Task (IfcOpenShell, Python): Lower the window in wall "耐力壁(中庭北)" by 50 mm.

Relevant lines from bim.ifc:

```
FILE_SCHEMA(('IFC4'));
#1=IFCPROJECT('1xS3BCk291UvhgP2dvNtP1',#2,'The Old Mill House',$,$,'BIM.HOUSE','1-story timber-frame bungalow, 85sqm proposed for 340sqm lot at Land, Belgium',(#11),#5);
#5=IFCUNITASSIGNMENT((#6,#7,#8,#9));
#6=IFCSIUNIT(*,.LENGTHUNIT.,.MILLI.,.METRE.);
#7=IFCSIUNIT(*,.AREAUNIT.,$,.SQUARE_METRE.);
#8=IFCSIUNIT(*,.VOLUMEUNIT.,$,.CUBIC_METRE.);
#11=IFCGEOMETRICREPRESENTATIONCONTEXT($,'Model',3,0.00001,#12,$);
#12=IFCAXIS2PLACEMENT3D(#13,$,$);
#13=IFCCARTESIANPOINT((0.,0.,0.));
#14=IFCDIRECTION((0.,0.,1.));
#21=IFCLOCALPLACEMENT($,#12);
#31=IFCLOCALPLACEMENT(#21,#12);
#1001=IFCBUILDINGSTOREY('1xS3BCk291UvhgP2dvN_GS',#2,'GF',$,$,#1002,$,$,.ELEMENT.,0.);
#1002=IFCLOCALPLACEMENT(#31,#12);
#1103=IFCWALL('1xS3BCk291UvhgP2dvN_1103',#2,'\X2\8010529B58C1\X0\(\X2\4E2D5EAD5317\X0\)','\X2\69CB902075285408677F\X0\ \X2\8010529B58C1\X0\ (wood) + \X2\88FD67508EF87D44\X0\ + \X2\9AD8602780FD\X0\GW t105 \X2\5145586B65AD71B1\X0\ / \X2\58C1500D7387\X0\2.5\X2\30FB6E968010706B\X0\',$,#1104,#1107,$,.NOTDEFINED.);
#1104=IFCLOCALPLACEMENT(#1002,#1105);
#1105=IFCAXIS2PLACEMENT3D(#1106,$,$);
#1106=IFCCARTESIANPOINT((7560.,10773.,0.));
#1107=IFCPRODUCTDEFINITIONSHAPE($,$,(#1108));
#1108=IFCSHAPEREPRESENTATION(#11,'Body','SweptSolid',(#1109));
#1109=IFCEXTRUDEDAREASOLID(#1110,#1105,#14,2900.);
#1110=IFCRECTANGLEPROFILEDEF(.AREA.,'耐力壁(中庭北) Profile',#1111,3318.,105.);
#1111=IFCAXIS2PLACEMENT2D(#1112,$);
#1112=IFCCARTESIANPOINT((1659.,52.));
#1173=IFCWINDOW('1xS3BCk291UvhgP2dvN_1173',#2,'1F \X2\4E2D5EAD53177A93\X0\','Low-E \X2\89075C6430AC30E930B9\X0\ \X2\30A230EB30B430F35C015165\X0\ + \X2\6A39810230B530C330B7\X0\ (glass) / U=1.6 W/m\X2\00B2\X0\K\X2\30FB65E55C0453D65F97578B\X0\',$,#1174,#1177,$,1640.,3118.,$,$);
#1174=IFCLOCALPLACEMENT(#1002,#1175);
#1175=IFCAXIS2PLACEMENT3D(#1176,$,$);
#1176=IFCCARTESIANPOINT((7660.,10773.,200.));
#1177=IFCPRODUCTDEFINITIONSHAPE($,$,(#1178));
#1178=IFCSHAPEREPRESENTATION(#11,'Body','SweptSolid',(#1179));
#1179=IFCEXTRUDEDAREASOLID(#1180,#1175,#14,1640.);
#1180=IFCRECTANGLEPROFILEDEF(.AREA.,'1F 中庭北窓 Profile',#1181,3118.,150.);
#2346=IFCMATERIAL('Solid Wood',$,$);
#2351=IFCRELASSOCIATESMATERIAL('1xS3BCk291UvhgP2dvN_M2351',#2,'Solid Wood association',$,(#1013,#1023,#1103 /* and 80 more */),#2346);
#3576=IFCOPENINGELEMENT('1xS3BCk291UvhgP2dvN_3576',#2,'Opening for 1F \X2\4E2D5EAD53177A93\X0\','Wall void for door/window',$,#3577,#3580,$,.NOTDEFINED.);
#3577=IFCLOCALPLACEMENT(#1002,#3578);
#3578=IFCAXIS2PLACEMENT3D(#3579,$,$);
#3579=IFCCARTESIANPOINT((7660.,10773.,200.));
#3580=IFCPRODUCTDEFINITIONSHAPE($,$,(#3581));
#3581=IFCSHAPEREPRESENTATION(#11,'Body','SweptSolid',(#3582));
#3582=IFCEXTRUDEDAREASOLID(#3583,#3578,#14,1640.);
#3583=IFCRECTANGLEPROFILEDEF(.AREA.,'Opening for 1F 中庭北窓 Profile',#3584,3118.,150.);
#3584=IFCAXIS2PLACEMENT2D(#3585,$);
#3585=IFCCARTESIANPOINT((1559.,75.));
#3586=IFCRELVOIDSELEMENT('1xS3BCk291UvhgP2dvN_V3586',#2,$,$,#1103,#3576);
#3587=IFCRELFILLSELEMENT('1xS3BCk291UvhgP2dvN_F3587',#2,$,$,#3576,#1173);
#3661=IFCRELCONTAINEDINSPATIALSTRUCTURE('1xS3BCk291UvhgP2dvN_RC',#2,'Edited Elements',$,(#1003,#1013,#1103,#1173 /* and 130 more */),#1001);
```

```python
import numpy as np
import ifcopenshell
import ifcopenshell.api.geometry
import ifcopenshell.util.placement
import ifcopenshell.util.unit

model = ifcopenshell.open("bim.ifc")
unit_scale = ifcopenshell.util.unit.calculate_unit_scale(model)

window = model.by_guid("1xS3BCk291UvhgP2dvN_1173")
opening = window.FillsVoids[0].RelatingOpeningElement
dz = -0.05 / unit_scale

shift = np.array([0.0, 0.0, dz])
# The window is not placed relative to its opening, so move both.
for product in (opening, window):
    matrix = ifcopenshell.util.placement.get_local_placement(product.ObjectPlacement)
    matrix[:3, 3] += shift
    ifcopenshell.api.geometry.edit_object_placement(model, product=product, matrix=matrix, is_si=False)

print(f"moved by {dz * unit_scale:+.3f} m")

model.write("bim_v2.ifc")
```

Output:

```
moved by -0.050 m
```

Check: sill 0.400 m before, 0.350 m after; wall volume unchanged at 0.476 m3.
